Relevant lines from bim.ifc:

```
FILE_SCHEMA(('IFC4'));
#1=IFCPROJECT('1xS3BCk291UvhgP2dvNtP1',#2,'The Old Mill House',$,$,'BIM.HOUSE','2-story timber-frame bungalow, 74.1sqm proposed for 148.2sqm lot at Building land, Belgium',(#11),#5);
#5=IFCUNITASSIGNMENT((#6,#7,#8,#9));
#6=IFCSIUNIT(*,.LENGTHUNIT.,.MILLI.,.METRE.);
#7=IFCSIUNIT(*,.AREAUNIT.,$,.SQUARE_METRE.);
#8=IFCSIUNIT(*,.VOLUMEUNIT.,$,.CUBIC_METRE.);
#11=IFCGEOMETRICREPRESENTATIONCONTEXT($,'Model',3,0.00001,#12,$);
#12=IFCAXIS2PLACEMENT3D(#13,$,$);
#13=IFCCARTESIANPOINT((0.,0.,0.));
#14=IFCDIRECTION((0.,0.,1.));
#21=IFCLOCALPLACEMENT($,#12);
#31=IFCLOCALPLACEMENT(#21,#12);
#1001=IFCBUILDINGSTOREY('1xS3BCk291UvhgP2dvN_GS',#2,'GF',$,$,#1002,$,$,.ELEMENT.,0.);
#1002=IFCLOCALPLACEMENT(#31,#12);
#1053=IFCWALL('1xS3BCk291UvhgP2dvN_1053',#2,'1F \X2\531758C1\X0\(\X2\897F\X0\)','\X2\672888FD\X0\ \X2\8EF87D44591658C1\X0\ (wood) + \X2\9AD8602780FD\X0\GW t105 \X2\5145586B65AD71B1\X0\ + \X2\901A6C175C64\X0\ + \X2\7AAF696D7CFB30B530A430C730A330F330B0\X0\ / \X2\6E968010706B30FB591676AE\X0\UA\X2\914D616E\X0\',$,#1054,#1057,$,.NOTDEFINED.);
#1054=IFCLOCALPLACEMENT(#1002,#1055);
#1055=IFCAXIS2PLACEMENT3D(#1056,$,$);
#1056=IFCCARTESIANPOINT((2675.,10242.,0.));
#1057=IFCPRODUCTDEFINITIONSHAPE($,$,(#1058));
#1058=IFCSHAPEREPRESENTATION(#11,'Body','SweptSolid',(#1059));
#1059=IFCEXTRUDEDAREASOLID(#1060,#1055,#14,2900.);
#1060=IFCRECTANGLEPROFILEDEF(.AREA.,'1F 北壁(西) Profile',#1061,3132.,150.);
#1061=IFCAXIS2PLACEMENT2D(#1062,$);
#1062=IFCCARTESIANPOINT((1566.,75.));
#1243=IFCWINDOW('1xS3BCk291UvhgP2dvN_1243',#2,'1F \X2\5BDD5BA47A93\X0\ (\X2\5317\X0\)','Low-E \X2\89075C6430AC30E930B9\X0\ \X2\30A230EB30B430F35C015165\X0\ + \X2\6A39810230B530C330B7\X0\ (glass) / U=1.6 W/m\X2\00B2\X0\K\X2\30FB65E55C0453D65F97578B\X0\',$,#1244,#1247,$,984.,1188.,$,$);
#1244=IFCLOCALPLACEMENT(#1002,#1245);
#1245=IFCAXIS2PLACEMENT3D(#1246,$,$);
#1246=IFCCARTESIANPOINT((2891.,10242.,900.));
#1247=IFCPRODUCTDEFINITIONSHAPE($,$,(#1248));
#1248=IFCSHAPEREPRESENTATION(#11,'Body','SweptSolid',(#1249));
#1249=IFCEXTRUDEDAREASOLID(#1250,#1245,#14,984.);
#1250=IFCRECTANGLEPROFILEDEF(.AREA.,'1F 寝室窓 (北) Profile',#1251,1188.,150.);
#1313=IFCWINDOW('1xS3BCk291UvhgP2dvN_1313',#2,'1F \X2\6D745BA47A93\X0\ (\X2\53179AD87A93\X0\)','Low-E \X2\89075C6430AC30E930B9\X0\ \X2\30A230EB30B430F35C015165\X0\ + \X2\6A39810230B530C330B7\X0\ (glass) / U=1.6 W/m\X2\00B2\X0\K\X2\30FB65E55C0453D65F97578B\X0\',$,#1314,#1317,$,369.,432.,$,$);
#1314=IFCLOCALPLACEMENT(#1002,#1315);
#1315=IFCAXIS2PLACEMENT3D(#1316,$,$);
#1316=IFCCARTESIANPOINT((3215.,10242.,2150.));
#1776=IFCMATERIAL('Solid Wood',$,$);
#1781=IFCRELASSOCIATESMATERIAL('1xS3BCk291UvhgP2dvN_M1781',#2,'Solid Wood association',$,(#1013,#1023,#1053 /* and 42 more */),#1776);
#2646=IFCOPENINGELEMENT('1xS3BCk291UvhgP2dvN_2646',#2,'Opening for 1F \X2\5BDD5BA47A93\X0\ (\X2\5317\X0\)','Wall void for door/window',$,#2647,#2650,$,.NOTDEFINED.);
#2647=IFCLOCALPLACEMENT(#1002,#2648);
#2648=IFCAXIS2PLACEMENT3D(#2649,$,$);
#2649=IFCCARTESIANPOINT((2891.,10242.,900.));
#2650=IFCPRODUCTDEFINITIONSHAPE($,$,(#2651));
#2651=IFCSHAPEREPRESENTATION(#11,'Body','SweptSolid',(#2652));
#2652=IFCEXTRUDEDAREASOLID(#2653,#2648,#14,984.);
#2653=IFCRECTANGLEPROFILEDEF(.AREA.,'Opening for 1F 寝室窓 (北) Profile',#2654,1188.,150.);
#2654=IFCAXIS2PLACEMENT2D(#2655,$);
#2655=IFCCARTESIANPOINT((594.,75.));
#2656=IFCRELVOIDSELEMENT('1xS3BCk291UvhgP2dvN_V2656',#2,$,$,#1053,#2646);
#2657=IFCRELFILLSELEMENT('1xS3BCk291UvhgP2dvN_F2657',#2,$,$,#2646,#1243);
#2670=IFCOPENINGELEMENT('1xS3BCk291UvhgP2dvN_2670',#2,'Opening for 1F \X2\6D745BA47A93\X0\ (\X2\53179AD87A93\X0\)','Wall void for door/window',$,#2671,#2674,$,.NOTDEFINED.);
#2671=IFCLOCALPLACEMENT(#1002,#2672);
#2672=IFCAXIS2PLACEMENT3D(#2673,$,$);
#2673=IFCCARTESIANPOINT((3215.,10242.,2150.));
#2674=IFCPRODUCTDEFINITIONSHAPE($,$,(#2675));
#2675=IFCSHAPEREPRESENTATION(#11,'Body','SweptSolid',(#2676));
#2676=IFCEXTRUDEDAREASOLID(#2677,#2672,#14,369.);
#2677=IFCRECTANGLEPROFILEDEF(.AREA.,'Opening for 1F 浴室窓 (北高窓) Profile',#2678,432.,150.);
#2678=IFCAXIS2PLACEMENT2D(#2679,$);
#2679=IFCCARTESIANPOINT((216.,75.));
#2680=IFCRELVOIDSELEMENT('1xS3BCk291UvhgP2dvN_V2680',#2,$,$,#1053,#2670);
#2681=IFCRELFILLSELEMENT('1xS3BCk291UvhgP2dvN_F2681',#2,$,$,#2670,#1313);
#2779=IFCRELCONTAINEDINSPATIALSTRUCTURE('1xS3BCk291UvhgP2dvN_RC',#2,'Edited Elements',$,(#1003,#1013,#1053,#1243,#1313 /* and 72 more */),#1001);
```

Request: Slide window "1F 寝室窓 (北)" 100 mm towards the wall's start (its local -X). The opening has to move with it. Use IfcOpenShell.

```python
import ifcopenshell
import ifcopenshell.api.geometry
import ifcopenshell.util.placement
import ifcopenshell.util.unit

model = ifcopenshell.open("bim.ifc")
unit_scale = ifcopenshell.util.unit.calculate_unit_scale(model)

window = model.by_guid("1xS3BCk291UvhgP2dvN_1243")
opening = window.FillsVoids[0].RelatingOpeningElement
wall = opening.VoidsElements[0].RelatingBuildingElement

wall_matrix = ifcopenshell.util.placement.get_local_placement(wall.ObjectPlacement)
shift = wall_matrix[:3, 0] * -0.1 / unit_scale
before = ifcopenshell.util.placement.get_local_placement(window.ObjectPlacement)[:3, 3].copy()

# The window is not placed relative to its opening, so move both.
for product in (opening, window):
    matrix = ifcopenshell.util.placement.get_local_placement(product.ObjectPlacement)
    matrix[:3, 3] += shift
    ifcopenshell.api.geometry.edit_object_placement(model, product=product, matrix=matrix, is_si=False)

after = ifcopenshell.util.placement.get_local_placement(window.ObjectPlacement)[:3, 3]
print("window moved by", (after - before).round(3) + 0.0)

model.write("bim_updated.ifc")
```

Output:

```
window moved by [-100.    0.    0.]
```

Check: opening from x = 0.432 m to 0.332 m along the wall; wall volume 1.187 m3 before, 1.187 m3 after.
